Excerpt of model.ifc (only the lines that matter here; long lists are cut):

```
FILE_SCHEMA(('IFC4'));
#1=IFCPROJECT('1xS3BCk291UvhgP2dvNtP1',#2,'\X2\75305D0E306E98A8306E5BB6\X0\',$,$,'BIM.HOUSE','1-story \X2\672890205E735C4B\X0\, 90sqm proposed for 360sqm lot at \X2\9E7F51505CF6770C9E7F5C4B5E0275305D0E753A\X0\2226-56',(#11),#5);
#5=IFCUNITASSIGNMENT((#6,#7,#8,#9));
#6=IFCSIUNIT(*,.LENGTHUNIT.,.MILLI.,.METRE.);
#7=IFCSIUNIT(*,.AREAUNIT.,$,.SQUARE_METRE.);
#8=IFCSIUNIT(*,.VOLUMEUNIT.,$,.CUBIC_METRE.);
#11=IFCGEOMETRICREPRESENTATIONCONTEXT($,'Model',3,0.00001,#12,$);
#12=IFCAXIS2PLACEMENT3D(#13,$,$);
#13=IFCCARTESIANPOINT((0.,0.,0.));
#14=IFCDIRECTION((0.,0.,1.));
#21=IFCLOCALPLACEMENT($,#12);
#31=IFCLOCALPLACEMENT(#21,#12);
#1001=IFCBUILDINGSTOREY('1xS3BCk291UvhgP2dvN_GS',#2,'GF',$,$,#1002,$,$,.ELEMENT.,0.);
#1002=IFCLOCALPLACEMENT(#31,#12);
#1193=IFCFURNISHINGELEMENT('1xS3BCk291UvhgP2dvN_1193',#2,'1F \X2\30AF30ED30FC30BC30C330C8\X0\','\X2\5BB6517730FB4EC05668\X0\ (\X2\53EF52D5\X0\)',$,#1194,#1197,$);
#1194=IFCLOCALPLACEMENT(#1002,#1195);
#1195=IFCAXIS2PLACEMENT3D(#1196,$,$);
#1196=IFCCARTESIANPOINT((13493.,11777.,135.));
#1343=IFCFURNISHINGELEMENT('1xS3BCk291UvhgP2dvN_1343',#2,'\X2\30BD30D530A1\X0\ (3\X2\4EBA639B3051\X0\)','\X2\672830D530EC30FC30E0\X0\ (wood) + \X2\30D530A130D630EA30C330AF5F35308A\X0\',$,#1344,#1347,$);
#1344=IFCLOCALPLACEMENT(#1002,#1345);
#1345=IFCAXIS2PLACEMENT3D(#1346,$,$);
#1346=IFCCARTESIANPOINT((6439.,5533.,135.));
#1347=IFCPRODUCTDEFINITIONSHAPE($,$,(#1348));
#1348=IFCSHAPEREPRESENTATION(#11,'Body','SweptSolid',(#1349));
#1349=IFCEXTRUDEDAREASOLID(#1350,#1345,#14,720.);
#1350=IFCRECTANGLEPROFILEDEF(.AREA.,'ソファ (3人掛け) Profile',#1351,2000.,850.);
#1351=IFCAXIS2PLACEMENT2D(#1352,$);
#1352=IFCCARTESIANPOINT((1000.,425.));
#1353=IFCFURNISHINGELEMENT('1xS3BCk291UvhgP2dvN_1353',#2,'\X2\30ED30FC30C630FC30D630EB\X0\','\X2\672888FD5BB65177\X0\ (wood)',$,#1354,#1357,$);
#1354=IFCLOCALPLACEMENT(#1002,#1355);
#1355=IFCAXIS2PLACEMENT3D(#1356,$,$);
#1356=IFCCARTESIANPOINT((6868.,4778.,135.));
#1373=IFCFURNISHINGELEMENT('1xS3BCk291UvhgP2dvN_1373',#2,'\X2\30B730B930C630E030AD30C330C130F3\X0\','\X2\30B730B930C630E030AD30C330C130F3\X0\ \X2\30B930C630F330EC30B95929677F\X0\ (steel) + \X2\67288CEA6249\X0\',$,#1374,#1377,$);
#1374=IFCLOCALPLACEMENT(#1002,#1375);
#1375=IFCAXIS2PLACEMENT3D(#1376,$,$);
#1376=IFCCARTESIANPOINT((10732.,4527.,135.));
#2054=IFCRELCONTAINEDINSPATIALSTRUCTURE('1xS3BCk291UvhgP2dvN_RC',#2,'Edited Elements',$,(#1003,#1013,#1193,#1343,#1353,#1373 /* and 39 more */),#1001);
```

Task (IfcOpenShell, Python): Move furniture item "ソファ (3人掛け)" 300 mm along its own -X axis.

```python
import ifcopenshell
import ifcopenshell.api.geometry
import ifcopenshell.util.placement
import ifcopenshell.util.unit

model = ifcopenshell.open("model.ifc")
unit_scale = ifcopenshell.util.unit.calculate_unit_scale(model)

item = model.by_guid("1xS3BCk291UvhgP2dvN_1343")
matrix = ifcopenshell.util.placement.get_local_placement(item.ObjectPlacement)
matrix[:3, 3] -= matrix[:3, 0] * 0.3 / unit_scale
ifcopenshell.api.geometry.edit_object_placement(model, product=item, matrix=matrix, is_si=False)

print(ifcopenshell.util.placement.get_local_placement(item.ObjectPlacement).round(3) + 0.0)

model.write("model_rev.ifc")
```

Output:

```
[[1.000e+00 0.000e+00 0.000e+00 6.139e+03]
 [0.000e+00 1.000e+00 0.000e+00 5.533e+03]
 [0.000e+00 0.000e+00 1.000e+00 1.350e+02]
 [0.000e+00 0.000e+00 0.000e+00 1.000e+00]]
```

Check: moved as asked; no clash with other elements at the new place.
